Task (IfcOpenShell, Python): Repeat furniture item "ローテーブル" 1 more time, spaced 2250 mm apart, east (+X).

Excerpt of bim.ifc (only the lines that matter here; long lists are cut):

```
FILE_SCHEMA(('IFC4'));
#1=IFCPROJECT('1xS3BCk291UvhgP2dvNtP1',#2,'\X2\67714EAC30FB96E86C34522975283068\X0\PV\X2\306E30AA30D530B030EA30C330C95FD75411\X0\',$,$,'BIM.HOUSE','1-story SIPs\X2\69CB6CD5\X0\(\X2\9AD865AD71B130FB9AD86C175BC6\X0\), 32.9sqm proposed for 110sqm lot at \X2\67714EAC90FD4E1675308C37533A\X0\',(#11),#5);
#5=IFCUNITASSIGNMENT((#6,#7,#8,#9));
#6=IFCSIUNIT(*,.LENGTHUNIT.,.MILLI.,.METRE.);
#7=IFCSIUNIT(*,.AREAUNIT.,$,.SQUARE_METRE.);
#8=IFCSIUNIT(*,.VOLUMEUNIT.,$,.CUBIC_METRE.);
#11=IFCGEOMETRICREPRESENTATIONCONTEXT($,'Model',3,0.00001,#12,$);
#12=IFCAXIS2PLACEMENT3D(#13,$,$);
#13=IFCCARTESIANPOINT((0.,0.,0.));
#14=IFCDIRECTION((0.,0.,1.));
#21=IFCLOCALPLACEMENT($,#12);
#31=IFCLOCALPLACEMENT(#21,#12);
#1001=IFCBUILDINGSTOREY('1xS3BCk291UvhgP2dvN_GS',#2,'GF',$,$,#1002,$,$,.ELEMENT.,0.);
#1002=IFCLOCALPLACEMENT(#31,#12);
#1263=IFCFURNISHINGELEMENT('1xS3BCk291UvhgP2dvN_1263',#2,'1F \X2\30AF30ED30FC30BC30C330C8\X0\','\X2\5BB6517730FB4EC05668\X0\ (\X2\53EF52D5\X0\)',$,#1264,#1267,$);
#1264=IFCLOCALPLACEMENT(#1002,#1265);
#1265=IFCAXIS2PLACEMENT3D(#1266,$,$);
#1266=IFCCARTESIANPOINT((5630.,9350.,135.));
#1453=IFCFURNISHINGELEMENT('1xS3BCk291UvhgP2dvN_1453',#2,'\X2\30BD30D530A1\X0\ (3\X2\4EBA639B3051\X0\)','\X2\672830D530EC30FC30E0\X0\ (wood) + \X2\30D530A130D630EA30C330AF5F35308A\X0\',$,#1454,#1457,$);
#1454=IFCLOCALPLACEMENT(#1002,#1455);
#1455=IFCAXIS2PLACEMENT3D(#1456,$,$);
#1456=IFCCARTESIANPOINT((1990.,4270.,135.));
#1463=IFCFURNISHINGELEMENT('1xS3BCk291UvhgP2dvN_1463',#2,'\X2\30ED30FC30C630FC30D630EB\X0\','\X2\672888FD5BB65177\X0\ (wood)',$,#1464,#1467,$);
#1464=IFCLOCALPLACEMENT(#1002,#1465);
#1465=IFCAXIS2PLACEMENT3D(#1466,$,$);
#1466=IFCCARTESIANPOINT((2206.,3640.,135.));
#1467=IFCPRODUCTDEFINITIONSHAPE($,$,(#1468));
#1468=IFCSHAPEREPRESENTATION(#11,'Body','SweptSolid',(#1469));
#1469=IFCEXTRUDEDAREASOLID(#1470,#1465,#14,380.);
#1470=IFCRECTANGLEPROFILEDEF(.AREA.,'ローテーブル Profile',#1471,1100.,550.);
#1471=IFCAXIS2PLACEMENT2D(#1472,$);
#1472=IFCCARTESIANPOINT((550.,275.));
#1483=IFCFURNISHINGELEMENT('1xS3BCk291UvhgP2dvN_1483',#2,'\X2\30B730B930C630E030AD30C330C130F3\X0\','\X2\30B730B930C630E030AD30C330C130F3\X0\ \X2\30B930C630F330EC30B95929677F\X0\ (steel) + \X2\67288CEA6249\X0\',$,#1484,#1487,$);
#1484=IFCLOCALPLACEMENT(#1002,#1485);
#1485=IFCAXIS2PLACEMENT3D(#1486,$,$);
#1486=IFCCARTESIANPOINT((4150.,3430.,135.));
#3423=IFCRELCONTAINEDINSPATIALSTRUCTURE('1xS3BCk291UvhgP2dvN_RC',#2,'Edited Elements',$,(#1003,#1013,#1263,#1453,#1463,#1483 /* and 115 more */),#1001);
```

```python
import numpy as np
import ifcopenshell
import ifcopenshell.api.geometry
import ifcopenshell.api.root
import ifcopenshell.util.element
import ifcopenshell.util.placement
import ifcopenshell.util.unit

model = ifcopenshell.open("bim.ifc")
unit_scale = ifcopenshell.util.unit.calculate_unit_scale(model)


def reuse_history(source, copy):
    """copy_class also copies each property set's owner history, people and application; keep the originals."""
    for rel in copy.IsDefinedBy:
        if rel.is_a("IfcRelDefinesByProperties") and (history := rel.RelatingPropertyDefinition.OwnerHistory):
            rel.RelatingPropertyDefinition.OwnerHistory = source.OwnerHistory
            ifcopenshell.util.element.remove_deep2(model, history)


source = model.by_guid("1xS3BCk291UvhgP2dvN_1463")
base = ifcopenshell.util.placement.get_local_placement(source.ObjectPlacement)
step = np.array([1.0, 0.0, 0.0]) * 2.25 / unit_scale

for i in range(1, 2):
    copy = ifcopenshell.api.root.copy_class(model, product=source)
    copy.Representation = ifcopenshell.util.element.copy_deep(
        model, source.Representation, exclude=["IfcGeometricRepresentationContext", "IfcRepresentationMap"]
    )
    reuse_history(source, copy)
    matrix = base.copy()
    matrix[:3, 3] += i * step
    print("added at", matrix[:3, 3].round(3) + 0.0)
    ifcopenshell.api.geometry.edit_object_placement(model, product=copy, matrix=matrix, is_si=False)

model.write("bim_v2.ifc")
```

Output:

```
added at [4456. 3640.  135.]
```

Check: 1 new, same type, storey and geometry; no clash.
